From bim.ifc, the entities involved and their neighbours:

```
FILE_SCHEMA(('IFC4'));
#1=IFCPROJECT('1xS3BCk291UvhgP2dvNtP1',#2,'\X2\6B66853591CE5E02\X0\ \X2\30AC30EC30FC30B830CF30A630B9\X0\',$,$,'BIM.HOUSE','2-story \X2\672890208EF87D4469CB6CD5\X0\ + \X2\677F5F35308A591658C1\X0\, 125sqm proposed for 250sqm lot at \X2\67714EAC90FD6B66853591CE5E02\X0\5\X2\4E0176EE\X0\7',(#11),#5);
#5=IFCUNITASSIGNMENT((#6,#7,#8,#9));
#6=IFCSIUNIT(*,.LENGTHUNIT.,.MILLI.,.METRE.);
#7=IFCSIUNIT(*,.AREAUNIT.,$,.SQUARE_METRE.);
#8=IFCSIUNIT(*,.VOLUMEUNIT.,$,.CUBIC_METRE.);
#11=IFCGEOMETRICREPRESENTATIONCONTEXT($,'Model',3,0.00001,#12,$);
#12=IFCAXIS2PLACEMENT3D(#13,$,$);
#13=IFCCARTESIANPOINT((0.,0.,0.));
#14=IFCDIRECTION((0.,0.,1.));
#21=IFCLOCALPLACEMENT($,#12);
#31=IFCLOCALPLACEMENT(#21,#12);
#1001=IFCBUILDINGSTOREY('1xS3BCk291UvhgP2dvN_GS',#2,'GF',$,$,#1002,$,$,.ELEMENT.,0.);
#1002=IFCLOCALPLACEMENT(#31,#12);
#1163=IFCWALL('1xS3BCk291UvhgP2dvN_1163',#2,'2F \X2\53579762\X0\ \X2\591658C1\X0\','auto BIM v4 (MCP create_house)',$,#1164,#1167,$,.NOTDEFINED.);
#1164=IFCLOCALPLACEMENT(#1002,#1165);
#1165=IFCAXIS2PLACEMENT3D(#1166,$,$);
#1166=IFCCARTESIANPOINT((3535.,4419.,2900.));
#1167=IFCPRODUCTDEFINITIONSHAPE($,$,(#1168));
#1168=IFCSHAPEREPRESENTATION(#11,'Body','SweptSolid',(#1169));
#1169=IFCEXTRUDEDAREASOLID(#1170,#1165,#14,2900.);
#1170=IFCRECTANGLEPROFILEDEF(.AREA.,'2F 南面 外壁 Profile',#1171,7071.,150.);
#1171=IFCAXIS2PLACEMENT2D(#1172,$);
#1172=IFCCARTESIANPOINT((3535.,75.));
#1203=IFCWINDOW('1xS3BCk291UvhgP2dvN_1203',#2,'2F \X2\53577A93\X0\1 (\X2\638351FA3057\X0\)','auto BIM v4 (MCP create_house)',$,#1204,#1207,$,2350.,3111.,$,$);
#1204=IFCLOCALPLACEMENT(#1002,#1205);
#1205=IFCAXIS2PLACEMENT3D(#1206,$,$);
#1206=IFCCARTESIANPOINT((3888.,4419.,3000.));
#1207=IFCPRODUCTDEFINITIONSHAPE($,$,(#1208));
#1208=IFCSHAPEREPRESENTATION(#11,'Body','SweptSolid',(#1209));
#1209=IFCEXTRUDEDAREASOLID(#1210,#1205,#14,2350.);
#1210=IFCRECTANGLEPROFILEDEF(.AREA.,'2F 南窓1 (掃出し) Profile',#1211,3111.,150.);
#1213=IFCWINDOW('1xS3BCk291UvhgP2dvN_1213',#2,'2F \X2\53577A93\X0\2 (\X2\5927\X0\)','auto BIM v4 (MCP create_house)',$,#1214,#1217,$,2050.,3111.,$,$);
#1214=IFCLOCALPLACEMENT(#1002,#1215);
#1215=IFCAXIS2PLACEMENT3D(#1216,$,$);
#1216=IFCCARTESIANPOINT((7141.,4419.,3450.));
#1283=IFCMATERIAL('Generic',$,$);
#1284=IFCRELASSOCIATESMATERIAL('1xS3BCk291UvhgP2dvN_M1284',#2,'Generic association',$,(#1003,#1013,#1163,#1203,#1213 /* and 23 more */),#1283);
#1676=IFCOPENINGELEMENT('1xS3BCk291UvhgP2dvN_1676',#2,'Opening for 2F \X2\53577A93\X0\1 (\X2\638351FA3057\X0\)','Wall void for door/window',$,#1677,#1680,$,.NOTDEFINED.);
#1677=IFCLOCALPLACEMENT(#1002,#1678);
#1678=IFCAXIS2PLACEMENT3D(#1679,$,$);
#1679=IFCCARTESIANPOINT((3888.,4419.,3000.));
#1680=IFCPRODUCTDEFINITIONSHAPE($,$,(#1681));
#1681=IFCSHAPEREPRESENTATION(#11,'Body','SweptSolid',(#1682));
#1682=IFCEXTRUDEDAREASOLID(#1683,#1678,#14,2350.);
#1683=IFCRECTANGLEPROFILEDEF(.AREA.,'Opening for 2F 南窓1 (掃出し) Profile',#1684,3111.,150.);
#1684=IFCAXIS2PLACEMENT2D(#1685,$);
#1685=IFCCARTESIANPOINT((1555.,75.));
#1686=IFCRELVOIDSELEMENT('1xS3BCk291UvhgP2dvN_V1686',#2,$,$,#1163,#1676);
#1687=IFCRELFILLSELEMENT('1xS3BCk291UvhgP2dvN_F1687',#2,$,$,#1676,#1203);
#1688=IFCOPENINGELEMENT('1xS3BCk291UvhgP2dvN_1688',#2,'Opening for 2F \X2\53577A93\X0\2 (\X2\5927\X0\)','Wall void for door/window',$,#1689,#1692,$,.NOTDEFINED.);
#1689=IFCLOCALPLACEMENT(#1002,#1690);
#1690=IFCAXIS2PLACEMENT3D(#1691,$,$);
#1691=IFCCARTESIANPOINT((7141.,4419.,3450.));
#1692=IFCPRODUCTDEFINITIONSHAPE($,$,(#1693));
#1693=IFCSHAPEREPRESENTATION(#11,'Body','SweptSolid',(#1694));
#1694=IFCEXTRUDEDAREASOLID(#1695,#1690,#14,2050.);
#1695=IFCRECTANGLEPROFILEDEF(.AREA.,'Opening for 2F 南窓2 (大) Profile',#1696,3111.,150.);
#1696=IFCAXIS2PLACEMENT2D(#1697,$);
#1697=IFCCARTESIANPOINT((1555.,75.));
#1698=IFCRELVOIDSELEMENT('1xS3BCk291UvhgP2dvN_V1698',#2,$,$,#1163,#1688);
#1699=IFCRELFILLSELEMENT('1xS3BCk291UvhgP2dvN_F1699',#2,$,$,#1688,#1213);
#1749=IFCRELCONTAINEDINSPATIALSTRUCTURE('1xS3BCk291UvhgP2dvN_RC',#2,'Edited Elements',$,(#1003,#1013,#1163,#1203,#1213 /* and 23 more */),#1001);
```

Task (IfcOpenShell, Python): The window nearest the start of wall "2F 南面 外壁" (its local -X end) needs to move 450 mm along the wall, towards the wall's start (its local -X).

```python
import ifcopenshell
import ifcopenshell.api.geometry
import ifcopenshell.util.placement
import ifcopenshell.util.unit

model = ifcopenshell.open("bim.ifc")
unit_scale = ifcopenshell.util.unit.calculate_unit_scale(model)

window = model.by_guid("1xS3BCk291UvhgP2dvN_1203")
opening = window.FillsVoids[0].RelatingOpeningElement
wall = opening.VoidsElements[0].RelatingBuildingElement

wall_matrix = ifcopenshell.util.placement.get_local_placement(wall.ObjectPlacement)
shift = wall_matrix[:3, 0] * -0.45 / unit_scale
before = ifcopenshell.util.placement.get_local_placement(window.ObjectPlacement)[:3, 3].copy()

# The window is not placed relative to its opening, so move both.
for product in (opening, window):
    matrix = ifcopenshell.util.placement.get_local_placement(product.ObjectPlacement)
    matrix[:3, 3] += shift
    ifcopenshell.api.geometry.edit_object_placement(model, product=product, matrix=matrix, is_si=False)

after = ifcopenshell.util.placement.get_local_placement(window.ObjectPlacement)[:3, 3]
print("window moved by", (after - before).round(3) + 0.0)

model.write("bim_v2.ifc")
```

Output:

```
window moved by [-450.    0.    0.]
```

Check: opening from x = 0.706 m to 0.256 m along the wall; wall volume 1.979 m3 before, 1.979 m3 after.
